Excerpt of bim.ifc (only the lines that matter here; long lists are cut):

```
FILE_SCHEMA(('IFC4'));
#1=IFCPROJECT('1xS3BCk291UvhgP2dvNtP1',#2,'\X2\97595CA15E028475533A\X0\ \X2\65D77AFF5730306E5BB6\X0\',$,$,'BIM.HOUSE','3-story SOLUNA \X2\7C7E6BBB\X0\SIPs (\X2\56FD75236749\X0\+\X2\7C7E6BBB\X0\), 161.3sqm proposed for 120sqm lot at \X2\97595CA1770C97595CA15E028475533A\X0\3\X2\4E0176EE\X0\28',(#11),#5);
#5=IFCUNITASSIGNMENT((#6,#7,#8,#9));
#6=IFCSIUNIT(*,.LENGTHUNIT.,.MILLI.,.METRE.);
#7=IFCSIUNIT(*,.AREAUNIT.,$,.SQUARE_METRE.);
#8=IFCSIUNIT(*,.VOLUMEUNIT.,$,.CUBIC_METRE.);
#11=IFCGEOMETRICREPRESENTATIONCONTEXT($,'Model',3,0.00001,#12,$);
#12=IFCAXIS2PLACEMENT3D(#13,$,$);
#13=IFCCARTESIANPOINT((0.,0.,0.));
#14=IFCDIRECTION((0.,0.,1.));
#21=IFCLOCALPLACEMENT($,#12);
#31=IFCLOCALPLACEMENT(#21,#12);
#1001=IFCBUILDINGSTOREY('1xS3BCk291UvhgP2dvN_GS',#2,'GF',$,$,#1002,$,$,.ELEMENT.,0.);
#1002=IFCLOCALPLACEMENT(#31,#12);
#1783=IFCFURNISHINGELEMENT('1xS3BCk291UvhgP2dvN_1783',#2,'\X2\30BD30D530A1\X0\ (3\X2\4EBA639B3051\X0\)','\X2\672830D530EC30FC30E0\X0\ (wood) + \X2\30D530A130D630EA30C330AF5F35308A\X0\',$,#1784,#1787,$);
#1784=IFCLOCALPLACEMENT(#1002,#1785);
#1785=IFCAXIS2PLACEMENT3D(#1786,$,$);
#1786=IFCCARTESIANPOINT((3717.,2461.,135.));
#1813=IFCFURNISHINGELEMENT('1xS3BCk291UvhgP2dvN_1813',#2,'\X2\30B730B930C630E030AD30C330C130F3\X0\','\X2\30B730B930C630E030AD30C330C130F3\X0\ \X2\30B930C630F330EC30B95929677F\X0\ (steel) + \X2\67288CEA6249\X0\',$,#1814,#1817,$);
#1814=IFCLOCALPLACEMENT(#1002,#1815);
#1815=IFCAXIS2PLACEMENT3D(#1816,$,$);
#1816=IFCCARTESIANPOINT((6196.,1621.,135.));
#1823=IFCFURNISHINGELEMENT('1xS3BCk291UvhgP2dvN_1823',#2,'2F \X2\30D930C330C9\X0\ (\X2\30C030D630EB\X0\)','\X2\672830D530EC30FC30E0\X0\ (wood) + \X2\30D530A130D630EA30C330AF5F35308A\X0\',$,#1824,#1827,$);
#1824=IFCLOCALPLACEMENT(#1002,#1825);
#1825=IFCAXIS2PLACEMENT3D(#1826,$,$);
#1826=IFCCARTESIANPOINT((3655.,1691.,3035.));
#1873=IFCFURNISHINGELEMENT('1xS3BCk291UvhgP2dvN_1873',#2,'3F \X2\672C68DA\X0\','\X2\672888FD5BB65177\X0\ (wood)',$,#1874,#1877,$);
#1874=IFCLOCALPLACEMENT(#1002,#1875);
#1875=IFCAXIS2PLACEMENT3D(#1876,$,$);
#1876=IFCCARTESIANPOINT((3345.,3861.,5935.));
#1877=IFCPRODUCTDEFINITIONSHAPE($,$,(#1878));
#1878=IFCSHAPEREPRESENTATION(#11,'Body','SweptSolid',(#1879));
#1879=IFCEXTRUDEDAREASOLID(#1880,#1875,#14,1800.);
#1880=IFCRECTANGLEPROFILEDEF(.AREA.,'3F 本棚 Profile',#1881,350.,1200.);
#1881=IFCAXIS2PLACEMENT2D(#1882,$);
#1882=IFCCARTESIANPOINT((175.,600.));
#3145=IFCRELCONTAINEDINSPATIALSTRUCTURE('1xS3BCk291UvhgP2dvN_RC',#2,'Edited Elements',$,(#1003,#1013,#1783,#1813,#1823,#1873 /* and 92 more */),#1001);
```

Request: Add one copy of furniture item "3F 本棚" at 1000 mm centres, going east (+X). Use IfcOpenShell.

```python
import numpy as np
import ifcopenshell
import ifcopenshell.api.geometry
import ifcopenshell.api.root
import ifcopenshell.util.element
import ifcopenshell.util.placement

model = ifcopenshell.open("bim.ifc")


def reuse_history(source, copy):
    """copy_class also copies each property set's owner history, people and application; keep the originals."""
    for rel in copy.IsDefinedBy:
        if rel.is_a("IfcRelDefinesByProperties") and (history := rel.RelatingPropertyDefinition.OwnerHistory):
            rel.RelatingPropertyDefinition.OwnerHistory = source.OwnerHistory
            ifcopenshell.util.element.remove_deep2(model, history)


source = model.by_id(1873)
base = ifcopenshell.util.placement.get_local_placement(source.ObjectPlacement)
step = np.array([1.0, 0.0, 0.0]) * 1000.0

for i in range(1, 2):
    copy = ifcopenshell.api.root.copy_class(model, product=source)
    copy.Representation = ifcopenshell.util.element.copy_deep(
        model, source.Representation, exclude=["IfcGeometricRepresentationContext", "IfcRepresentationMap"]
    )
    reuse_history(source, copy)
    matrix = base.copy()
    matrix[:3, 3] += i * step
    print("added at", matrix[:3, 3].round(3) + 0.0)
    ifcopenshell.api.geometry.edit_object_placement(model, product=copy, matrix=matrix, is_si=False)

model.write("bim_rev.ifc")
```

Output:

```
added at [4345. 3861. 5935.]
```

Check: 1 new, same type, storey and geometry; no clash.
